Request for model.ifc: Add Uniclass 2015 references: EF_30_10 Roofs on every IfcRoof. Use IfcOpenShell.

First a look at what the model holds.

```python
import ifcopenshell

model = ifcopenshell.open("model.ifc")
print(model.schema)
print("classifications:", [c.Name for c in model.by_type("IfcClassification")])
for ifc_class in ("IfcDoor", "IfcRoof", "IfcStair", "IfcWall", "IfcWindow"):
    print(ifc_class, len(model.by_type(ifc_class)))
```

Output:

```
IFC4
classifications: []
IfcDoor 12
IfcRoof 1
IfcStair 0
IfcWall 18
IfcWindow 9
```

```python
import ifcopenshell
import ifcopenshell.api.classification

model = ifcopenshell.open("model.ifc")

system = ifcopenshell.api.classification.add_classification(model, classification="Uniclass 2015")

codes = {
    "IfcRoof": ("EF_30_10", "Roofs"),
}
for ifc_class, (code, name) in codes.items():
    products = model.by_type(ifc_class)
    ifcopenshell.api.classification.add_reference(
        model, products=products, classification=system, identification=code, name=name
    )
    print(code, len(products))

model.write("model_edited.ifc")
```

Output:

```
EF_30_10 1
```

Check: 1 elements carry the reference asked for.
